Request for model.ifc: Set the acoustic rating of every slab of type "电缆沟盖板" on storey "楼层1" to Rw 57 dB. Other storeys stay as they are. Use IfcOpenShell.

First a look at what the model holds.

```python
import ifcopenshell
import ifcopenshell.util.element

model = ifcopenshell.open("model.ifc")
print(model.schema)
storey = next(s for s in model.by_type("IfcBuildingStorey") if s.Name == "楼层1")
slabs = [e for e in ifcopenshell.util.element.get_decomposition(storey) if e.is_a("IfcSlab")]
seen = {}
for e in slabs:
    element_type = ifcopenshell.util.element.get_type(e)
    key = (element_type.Name if element_type != e and element_type else None, ifcopenshell.util.element.get_pset(e, "Pset_SlabCommon", "AcousticRating"))
    seen[key] = seen.get(key, 0) + 1
for (name, value), count in sorted(seen.items(), key=str):
    print(count, "x", name, "|", value)
```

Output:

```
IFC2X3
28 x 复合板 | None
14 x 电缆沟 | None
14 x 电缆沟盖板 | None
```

```python
import ifcopenshell
import ifcopenshell.api.pset
import ifcopenshell.util.element

model = ifcopenshell.open("model.ifc")

storey = next(s for s in model.by_type("IfcBuildingStorey") if s.Name == "楼层1")
slabs = [e for e in ifcopenshell.util.element.get_decomposition(storey) if e.is_a("IfcSlab")]

count = 0
for e in slabs:
    element_type = ifcopenshell.util.element.get_type(e)
    if element_type in (None, e) or element_type.Name != "电缆沟盖板":
        continue
    # add_pset returns the element's existing set when there is one.
    pset = ifcopenshell.api.pset.add_pset(model, product=e, name="Pset_SlabCommon")
    ifcopenshell.api.pset.edit_pset(model, pset=pset, properties={"AcousticRating": "Rw 57 dB"})
    count += 1

print(count, "slabs updated")

model.write("model_v2.ifc")
```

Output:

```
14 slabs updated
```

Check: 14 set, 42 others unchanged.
